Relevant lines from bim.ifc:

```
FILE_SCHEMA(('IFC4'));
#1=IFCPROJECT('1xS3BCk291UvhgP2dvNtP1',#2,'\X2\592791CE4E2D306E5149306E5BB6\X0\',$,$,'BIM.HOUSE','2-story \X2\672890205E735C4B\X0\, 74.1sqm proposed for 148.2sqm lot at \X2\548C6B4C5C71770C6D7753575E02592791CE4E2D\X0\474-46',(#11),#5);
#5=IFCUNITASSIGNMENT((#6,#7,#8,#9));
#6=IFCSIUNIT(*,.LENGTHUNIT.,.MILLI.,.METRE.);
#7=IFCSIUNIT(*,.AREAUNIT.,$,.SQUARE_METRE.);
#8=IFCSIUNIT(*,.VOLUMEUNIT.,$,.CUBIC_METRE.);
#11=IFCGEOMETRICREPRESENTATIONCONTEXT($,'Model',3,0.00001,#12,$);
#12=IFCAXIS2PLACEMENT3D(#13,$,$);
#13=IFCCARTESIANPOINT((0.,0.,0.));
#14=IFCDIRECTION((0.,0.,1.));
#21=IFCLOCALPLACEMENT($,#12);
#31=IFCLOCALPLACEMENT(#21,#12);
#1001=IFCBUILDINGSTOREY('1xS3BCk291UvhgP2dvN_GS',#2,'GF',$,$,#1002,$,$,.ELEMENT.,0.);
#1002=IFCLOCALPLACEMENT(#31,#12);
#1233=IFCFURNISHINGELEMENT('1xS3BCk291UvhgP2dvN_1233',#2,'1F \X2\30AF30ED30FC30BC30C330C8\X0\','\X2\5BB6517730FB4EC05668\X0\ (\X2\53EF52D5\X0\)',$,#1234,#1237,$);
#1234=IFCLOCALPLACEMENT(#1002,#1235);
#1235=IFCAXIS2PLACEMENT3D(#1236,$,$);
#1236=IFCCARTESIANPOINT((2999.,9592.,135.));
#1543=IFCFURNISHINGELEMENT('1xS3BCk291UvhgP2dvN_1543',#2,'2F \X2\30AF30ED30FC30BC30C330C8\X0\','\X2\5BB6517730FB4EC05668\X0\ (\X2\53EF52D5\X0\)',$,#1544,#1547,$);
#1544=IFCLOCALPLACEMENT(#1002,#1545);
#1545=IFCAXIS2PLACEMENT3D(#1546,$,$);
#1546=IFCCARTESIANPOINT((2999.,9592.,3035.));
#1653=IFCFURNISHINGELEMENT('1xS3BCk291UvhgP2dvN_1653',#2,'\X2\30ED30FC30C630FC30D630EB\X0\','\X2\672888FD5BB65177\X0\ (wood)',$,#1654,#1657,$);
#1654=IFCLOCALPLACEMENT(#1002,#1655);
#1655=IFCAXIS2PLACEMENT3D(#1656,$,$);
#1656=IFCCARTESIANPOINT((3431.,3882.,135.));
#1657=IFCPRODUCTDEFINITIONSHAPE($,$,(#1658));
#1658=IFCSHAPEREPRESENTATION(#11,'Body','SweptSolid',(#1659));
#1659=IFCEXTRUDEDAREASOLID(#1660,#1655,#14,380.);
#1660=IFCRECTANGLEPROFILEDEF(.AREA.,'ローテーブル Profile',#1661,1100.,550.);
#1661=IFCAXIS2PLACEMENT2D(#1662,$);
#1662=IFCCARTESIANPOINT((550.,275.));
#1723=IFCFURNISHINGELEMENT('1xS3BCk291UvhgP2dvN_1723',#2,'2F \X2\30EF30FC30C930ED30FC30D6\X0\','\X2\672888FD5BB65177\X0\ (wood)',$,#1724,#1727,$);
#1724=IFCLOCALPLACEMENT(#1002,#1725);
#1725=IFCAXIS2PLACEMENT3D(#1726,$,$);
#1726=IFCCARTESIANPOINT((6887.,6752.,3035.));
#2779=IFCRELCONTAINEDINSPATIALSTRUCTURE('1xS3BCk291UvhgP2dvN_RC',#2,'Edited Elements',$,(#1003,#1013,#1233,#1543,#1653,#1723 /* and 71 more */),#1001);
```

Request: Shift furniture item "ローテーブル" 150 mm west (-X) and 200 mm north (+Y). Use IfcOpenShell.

```python
import ifcopenshell
import ifcopenshell.api.geometry
import ifcopenshell.util.placement

model = ifcopenshell.open("bim.ifc")

item = model.by_guid("1xS3BCk291UvhgP2dvN_1653")
matrix = ifcopenshell.util.placement.get_local_placement(item.ObjectPlacement)
matrix[0, 3] -= 150.0
matrix[1, 3] += 200.0
ifcopenshell.api.geometry.edit_object_placement(model, product=item, matrix=matrix, is_si=False)

print(ifcopenshell.util.placement.get_local_placement(item.ObjectPlacement).round(3) + 0.0)

model.write("bim_rev.ifc")
```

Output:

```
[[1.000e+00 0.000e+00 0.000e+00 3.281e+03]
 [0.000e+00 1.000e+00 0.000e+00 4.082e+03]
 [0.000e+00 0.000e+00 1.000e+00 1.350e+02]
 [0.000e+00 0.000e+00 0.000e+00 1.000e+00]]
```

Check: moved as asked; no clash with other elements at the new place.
